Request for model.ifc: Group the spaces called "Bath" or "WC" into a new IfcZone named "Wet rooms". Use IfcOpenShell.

First a look at what the model holds.

```python
import ifcopenshell

model = ifcopenshell.open("model.ifc")
print(model.schema)
seen = {}
for space in model.by_type("IfcSpace"):
    seen[space.LongName] = seen.get(space.LongName, 0) + 1
for name, count in sorted(seen.items(), key=str):
    print(count, "x", name)
print("zones:", [z.Name for z in model.by_type("IfcZone")][:20])
```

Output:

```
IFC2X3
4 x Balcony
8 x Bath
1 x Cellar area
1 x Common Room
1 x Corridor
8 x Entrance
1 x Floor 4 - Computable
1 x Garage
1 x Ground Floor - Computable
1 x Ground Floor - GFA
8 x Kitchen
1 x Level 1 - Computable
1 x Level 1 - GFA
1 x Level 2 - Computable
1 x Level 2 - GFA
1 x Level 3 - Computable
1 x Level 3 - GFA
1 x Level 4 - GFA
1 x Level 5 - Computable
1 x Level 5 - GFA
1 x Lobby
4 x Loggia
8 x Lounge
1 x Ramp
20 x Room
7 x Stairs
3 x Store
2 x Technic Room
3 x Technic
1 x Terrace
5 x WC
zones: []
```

```python
import ifcopenshell
import ifcopenshell.api.group
import ifcopenshell.api.root

model = ifcopenshell.open("model.ifc")

names = {"Bath", "WC"}
spaces = [s for s in model.by_type("IfcSpace") if s.LongName in names]

zone = ifcopenshell.api.root.create_entity(model, ifc_class="IfcZone", name="Wet rooms")
ifcopenshell.api.group.assign_group(model, products=spaces, group=zone)
print(len(spaces), "spaces in", zone.Name)

model.write("model_updated.ifc")
```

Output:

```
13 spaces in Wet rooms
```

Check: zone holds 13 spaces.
